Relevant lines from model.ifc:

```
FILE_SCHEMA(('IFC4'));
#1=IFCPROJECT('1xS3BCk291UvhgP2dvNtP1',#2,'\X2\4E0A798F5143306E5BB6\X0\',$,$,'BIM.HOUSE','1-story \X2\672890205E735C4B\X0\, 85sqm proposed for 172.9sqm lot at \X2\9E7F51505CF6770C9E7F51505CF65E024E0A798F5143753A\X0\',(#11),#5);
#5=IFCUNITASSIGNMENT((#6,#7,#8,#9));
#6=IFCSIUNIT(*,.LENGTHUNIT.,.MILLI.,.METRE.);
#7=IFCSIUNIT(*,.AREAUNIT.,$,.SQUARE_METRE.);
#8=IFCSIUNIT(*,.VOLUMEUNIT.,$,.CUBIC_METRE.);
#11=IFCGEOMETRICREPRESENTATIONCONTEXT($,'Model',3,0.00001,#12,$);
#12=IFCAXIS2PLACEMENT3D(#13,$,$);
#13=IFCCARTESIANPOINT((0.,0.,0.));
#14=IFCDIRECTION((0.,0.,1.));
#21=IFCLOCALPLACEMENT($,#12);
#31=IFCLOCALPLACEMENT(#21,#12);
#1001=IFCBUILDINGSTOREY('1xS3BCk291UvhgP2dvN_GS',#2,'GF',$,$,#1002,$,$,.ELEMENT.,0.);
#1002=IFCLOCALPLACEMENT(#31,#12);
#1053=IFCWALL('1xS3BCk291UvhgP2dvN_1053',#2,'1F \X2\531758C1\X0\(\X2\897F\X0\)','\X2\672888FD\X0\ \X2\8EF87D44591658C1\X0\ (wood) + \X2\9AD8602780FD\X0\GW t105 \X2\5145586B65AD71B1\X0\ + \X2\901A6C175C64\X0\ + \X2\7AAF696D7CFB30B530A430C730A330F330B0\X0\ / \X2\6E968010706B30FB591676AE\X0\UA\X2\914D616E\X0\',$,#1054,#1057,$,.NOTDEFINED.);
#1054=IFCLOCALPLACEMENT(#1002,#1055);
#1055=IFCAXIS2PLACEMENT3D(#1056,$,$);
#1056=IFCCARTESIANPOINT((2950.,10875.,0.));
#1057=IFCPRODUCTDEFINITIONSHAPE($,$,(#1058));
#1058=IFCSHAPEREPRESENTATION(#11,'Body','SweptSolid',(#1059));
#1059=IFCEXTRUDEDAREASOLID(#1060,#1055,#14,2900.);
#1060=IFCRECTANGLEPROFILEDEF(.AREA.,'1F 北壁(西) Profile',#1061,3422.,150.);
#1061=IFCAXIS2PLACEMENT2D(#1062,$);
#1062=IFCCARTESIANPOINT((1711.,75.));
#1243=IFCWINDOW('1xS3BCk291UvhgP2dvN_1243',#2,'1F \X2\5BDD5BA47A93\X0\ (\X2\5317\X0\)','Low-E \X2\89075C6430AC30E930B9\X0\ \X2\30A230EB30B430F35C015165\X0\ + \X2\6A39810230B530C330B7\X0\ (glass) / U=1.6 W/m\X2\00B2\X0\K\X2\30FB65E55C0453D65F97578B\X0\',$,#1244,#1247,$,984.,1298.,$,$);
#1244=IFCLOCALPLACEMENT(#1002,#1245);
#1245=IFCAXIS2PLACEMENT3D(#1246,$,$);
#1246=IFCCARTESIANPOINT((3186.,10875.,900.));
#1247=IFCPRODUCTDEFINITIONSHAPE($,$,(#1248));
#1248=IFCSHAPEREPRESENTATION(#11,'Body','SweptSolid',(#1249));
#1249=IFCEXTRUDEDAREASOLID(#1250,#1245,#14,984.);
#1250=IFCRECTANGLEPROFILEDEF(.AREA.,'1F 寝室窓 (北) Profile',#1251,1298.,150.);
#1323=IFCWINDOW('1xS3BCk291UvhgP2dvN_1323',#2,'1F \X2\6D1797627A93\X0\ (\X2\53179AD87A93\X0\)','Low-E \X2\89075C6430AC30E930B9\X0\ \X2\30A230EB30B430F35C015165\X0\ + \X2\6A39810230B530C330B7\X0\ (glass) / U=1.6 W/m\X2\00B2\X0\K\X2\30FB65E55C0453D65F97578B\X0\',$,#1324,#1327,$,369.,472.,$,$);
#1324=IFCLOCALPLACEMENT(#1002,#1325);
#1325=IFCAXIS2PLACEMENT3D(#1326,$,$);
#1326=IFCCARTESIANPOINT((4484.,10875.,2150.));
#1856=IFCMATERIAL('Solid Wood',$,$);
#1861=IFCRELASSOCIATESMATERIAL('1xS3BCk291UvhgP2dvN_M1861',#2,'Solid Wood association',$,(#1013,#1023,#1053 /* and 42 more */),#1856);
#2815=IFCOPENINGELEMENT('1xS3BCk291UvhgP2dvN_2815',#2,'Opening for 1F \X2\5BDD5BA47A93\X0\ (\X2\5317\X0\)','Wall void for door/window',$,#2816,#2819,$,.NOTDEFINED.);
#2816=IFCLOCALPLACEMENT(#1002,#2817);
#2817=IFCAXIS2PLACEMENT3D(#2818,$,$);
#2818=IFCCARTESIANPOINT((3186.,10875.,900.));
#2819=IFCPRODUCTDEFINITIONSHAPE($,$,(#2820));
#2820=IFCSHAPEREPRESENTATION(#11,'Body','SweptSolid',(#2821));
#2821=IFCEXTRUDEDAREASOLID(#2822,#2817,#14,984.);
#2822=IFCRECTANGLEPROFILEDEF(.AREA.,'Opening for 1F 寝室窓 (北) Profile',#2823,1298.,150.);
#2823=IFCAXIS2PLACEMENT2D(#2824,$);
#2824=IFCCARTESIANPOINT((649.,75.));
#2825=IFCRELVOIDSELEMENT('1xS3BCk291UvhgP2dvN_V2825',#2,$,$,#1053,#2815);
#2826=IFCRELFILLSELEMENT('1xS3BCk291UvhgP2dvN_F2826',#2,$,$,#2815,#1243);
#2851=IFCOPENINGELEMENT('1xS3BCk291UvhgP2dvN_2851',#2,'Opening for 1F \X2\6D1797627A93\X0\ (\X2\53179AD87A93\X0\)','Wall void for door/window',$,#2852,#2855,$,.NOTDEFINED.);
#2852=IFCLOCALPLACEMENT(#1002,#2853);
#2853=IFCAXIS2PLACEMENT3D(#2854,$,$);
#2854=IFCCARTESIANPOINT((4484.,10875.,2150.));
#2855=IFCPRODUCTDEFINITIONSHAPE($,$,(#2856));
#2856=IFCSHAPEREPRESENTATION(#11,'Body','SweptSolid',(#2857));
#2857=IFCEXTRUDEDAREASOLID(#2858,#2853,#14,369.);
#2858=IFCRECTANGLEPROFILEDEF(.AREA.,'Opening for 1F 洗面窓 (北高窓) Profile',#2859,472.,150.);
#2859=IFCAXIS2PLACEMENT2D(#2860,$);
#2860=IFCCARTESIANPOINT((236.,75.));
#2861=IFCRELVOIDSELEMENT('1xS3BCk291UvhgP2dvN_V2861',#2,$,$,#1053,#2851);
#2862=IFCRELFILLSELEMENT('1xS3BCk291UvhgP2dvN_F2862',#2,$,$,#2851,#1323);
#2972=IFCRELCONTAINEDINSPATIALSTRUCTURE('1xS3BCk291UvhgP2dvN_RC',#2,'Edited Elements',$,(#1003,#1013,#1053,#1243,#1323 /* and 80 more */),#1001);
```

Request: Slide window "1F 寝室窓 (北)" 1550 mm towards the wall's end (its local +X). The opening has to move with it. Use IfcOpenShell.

```python
import ifcopenshell
import ifcopenshell.api.geometry
import ifcopenshell.util.placement

model = ifcopenshell.open("model.ifc")

window = model.by_guid("1xS3BCk291UvhgP2dvN_1243")
opening = window.FillsVoids[0].RelatingOpeningElement
wall = opening.VoidsElements[0].RelatingBuildingElement

wall_matrix = ifcopenshell.util.placement.get_local_placement(wall.ObjectPlacement)
shift = wall_matrix[:3, 0] * 1550.0
before = ifcopenshell.util.placement.get_local_placement(window.ObjectPlacement)[:3, 3].copy()

# The window is not placed relative to its opening, so move both.
for product in (opening, window):
    matrix = ifcopenshell.util.placement.get_local_placement(product.ObjectPlacement)
    matrix[:3, 3] += shift
    ifcopenshell.api.geometry.edit_object_placement(model, product=product, matrix=matrix, is_si=False)

after = ifcopenshell.util.placement.get_local_placement(window.ObjectPlacement)[:3, 3]
print("window moved by", (after - before).round(3) + 0.0)

model.write("model_rev.ifc")
```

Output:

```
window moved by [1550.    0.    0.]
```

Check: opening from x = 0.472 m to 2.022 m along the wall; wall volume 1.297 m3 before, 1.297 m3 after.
